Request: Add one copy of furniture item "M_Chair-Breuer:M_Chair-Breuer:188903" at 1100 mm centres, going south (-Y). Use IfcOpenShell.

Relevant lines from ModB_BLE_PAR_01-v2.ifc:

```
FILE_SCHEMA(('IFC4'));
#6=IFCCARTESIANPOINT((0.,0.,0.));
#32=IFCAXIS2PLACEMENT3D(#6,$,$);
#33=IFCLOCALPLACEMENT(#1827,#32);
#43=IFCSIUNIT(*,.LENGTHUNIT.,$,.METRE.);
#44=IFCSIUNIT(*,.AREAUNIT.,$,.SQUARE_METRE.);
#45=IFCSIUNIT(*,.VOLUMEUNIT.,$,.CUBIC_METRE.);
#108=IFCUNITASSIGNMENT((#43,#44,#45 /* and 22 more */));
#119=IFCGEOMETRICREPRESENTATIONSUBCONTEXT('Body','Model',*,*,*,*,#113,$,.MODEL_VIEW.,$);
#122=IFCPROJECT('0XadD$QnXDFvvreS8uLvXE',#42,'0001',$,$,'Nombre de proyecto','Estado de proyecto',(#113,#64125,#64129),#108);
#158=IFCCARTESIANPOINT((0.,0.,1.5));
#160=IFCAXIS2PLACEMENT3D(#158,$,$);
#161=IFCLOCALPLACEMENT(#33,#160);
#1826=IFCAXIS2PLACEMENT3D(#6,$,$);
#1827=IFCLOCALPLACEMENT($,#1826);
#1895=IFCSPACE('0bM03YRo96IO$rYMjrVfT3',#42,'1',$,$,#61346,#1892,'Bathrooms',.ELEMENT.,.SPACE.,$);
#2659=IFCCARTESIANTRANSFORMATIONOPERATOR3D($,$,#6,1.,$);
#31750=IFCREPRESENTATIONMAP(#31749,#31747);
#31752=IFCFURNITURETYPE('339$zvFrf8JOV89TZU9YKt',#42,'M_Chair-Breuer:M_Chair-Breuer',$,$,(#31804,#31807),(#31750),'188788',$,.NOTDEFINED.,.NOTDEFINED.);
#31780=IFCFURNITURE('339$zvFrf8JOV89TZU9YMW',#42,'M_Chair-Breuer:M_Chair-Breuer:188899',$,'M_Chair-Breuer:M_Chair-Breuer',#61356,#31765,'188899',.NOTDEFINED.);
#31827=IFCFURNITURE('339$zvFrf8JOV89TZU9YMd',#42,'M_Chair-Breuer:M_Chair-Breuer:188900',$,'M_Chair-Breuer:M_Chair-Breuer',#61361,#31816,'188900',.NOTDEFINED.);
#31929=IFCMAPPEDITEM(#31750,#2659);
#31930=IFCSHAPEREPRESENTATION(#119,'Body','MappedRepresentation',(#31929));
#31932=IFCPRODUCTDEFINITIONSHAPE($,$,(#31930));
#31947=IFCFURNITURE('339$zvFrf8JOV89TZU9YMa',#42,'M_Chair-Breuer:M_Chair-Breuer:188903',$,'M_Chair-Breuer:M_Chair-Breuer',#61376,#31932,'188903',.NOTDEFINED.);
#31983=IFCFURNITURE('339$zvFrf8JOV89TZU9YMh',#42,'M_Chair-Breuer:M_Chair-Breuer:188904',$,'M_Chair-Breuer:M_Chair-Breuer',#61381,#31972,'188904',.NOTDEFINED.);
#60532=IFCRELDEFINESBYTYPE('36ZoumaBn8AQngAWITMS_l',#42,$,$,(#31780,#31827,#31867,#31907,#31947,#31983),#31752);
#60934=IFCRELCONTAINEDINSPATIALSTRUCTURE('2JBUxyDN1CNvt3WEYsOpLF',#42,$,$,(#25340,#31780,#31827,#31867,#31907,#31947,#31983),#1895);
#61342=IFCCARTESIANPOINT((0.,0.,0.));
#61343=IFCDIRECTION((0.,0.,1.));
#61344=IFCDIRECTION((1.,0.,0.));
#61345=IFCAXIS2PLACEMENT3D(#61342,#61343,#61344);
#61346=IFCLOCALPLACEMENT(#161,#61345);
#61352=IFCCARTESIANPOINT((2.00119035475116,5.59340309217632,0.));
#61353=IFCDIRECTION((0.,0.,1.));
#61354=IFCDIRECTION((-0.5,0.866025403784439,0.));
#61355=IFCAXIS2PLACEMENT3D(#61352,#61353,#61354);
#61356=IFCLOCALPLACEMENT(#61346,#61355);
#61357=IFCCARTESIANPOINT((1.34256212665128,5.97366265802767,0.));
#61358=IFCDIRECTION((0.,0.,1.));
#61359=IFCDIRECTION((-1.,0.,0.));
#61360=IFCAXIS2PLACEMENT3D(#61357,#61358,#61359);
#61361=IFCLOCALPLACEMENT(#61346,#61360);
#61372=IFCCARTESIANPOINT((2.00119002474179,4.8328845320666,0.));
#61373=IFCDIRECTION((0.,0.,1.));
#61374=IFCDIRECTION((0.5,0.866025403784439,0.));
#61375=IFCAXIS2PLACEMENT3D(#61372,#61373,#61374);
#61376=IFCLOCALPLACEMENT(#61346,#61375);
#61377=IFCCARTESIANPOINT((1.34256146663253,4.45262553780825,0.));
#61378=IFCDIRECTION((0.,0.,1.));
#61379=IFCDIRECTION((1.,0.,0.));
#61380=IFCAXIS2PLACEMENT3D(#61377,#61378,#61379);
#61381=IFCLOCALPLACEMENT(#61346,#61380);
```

```python
import numpy as np
import ifcopenshell
import ifcopenshell.api.geometry
import ifcopenshell.api.root
import ifcopenshell.util.element
import ifcopenshell.util.placement

model = ifcopenshell.open("ModB_BLE_PAR_01-v2.ifc")


def reuse_history(source, copy):
    """copy_class also copies each property set's owner history, people and application; keep the originals."""
    for rel in copy.IsDefinedBy:
        if rel.is_a("IfcRelDefinesByProperties") and (history := rel.RelatingPropertyDefinition.OwnerHistory):
            rel.RelatingPropertyDefinition.OwnerHistory = source.OwnerHistory
            ifcopenshell.util.element.remove_deep2(model, history)


source = model.by_guid("339$zvFrf8JOV89TZU9YMa")
base = ifcopenshell.util.placement.get_local_placement(source.ObjectPlacement)
step = np.array([0.0, -1.0, 0.0]) * 1.1

for i in range(1, 2):
    copy = ifcopenshell.api.root.copy_class(model, product=source)
    copy.Representation = ifcopenshell.util.element.copy_deep(
        model, source.Representation, exclude=["IfcGeometricRepresentationContext", "IfcRepresentationMap"]
    )
    copy.Name = "M_Chair-Breuer:M_Chair-Breuer"
    copy.Tag = None
    reuse_history(source, copy)
    matrix = base.copy()
    matrix[:3, 3] += i * step
    print("added at", matrix[:3, 3].round(3) + 0.0)
    ifcopenshell.api.geometry.edit_object_placement(model, product=copy, matrix=matrix, is_si=False)

model.write("ModB_BLE_PAR_01-v2-out.ifc")
```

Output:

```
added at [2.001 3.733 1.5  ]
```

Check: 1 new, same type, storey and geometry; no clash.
